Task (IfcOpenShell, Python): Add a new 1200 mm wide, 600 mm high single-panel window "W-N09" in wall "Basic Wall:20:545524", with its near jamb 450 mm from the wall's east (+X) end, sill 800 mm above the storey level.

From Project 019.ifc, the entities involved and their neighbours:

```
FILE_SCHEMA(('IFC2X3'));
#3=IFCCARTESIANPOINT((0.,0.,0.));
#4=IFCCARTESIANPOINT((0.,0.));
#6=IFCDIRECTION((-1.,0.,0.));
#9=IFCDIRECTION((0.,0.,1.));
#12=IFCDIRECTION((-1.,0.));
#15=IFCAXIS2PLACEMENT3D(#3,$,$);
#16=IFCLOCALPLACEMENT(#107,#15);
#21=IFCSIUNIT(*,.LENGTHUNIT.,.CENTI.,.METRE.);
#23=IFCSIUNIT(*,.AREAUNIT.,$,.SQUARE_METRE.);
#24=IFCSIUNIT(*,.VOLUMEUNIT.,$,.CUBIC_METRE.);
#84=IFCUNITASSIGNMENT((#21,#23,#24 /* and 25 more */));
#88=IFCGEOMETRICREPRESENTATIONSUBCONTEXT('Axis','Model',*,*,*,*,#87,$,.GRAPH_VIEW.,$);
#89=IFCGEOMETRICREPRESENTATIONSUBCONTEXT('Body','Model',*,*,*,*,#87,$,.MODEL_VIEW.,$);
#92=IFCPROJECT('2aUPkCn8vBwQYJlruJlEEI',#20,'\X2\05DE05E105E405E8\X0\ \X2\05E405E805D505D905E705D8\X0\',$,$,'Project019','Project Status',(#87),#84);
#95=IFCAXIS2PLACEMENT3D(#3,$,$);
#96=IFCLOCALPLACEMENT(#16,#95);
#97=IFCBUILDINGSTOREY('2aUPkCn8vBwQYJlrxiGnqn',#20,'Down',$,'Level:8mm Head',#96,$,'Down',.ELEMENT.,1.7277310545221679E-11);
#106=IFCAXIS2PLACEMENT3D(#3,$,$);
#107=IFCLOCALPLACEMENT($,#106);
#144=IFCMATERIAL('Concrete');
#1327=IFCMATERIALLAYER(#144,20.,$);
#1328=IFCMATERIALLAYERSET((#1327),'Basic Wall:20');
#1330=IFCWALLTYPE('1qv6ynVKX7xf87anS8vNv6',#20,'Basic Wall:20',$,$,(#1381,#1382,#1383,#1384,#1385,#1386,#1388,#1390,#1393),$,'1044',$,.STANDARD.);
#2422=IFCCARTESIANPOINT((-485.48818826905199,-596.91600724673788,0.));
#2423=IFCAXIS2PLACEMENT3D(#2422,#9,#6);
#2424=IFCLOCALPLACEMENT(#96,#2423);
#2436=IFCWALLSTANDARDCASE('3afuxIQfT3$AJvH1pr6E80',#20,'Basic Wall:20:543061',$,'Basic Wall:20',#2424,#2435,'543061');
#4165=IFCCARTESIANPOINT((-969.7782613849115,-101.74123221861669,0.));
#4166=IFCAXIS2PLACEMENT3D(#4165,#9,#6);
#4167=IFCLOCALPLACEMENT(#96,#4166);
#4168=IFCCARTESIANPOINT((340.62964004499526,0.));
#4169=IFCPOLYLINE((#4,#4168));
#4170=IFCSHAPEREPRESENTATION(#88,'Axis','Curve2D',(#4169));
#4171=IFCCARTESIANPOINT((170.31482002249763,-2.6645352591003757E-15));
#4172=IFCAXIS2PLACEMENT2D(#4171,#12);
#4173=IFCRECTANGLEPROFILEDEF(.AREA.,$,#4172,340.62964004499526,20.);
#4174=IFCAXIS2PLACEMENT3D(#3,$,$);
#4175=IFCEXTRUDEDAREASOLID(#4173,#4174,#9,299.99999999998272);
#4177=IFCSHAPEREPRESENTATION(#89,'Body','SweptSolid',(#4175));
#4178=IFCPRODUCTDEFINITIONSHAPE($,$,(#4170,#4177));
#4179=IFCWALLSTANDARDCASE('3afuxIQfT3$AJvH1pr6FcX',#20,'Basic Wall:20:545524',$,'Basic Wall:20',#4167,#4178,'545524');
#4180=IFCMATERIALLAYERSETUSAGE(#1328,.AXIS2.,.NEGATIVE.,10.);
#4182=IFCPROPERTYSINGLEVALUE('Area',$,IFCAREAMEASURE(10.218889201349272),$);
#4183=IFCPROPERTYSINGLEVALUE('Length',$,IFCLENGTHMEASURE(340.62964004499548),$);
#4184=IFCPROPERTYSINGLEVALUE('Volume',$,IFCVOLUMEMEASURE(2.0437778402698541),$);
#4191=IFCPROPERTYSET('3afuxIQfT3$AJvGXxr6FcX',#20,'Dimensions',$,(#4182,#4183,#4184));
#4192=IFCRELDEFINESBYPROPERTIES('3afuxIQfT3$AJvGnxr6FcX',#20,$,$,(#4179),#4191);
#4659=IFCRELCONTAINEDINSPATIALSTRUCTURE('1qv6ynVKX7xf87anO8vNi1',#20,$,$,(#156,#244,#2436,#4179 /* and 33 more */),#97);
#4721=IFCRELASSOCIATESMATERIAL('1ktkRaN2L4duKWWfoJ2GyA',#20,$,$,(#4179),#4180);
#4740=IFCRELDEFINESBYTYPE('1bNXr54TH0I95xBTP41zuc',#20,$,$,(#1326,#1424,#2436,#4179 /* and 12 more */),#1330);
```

```python
import numpy as np
import ifcopenshell
import ifcopenshell.api.feature
import ifcopenshell.api.geometry
import ifcopenshell.api.pset
import ifcopenshell.api.root
import ifcopenshell.api.spatial
import ifcopenshell.api.type
import ifcopenshell.geom
import ifcopenshell.util.element
import ifcopenshell.util.placement
import ifcopenshell.util.representation
import ifcopenshell.util.shape
import ifcopenshell.util.unit

model = ifcopenshell.open("Project 019.ifc")
unit_scale = ifcopenshell.util.unit.calculate_unit_scale(model)
area_scale = ifcopenshell.util.unit.calculate_unit_scale(model, "AREAUNIT")
volume_scale = ifcopenshell.util.unit.calculate_unit_scale(model, "VOLUMEUNIT")
settings = ifcopenshell.geom.settings()


def volume(element):
    """Net volume in cubic metres, openings subtracted."""
    shape = ifcopenshell.geom.create_shape(settings, element)
    return ifcopenshell.util.shape.get_volume(shape.geometry)


wall = model.by_id(4179)
storey = ifcopenshell.util.element.get_container(wall, ifc_class="IfcBuildingStorey")
context = ifcopenshell.util.representation.get_context(model, "Model", "Body", "MODEL_VIEW")
before = volume(wall)

width, height, from_end, sill = 1.2, 0.6, 0.45, 0.8  # metres

# The wall runs along its own X axis, and the end named is its -X end.
wall_shape = ifcopenshell.geom.create_shape(settings, wall)
x, y, z = ifcopenshell.util.shape.get_vertices(wall_shape.geometry).T
start = x.min() + from_end
face, thickness = float(y.min()), float(y.max() - y.min())
wall_matrix = ifcopenshell.util.placement.get_local_placement(wall.ObjectPlacement)
level = ifcopenshell.util.placement.get_local_placement(storey.ObjectPlacement)[2, 3]


def in_wall(x, y):
    """Placement at x, y metres in the wall's axes, at sill height."""
    matrix = wall_matrix.copy()
    matrix[:, 3] = wall_matrix @ np.array([x / unit_scale, y / unit_scale, 0.0, 1.0])
    matrix[2, 3] = level + sill / unit_scale
    return matrix


# Opening: a box that overshoots both wall faces by 50 mm.
opening = ifcopenshell.api.root.create_entity(model, ifc_class="IfcOpeningElement")
box = ifcopenshell.api.geometry.add_wall_representation(
    model, context=context, length=width, height=height, thickness=thickness + 0.1
)
ifcopenshell.api.geometry.assign_representation(model, product=opening, representation=box)
ifcopenshell.api.geometry.edit_object_placement(model, product=opening, matrix=in_wall(start, face - 0.05), is_si=False)
ifcopenshell.api.feature.add_feature(model, feature=opening, element=wall)

window = ifcopenshell.api.root.create_entity(model, ifc_class="IfcWindow", name="W-N09")
window.OverallWidth, window.OverallHeight = width / unit_scale, height / unit_scale
body = ifcopenshell.api.geometry.add_window_representation(
    model,
    context=context,
    overall_width=window.OverallWidth,
    overall_height=window.OverallHeight,
    partition_type="SINGLE_PANEL",
)
ifcopenshell.api.geometry.assign_representation(model, product=window, representation=body)
ifcopenshell.api.spatial.assign_container(model, products=[window], relating_structure=storey)
fills = ifcopenshell.api.feature.add_filling(model, opening=opening, element=window)
fills.OwnerHistory = window.OwnerHistory  # required in IFC2X3

# IFC2X3 keeps the operation on the window style.
style = ifcopenshell.api.root.create_entity(model, ifc_class="IfcWindowStyle", name="W-N09")
style.OperationType, style.ConstructionType = "SINGLE_PANEL", "NOTDEFINED"
style.ParameterTakesPrecedence = style.Sizeable = False
ifcopenshell.api.type.assign_type(model, related_objects=[window], relating_type=style)

# Centre the window in the wall's thickness.
ifcopenshell.api.geometry.edit_object_placement(model, product=window, matrix=in_wall(start, face), is_si=False)
window_shape = ifcopenshell.geom.create_shape(settings, window)
depth = ifcopenshell.util.shape.get_vertices(window_shape.geometry)[:, 1]
offset = face + thickness / 2 - (depth.min() + depth.max()) / 2
ifcopenshell.api.geometry.edit_object_placement(model, product=window, matrix=in_wall(start, offset), is_si=False)

after = volume(wall)

# Update the wall's stored quantities.
pset = model.by_id(ifcopenshell.util.element.get_pset(wall, "Dimensions", should_inherit=False)["id"])
ifcopenshell.api.pset.edit_pset(model, pset=pset, properties={
    "Area": model.create_entity("IfcAreaMeasure", after / thickness / area_scale),
    "Volume": model.create_entity("IfcVolumeMeasure", after / volume_scale),
})

print(f"wall volume {before:.3f} -> {after:.3f} m3")

model.write("Project 019-out.ifc")
```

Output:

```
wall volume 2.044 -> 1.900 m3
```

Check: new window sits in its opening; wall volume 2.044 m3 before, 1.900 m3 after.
